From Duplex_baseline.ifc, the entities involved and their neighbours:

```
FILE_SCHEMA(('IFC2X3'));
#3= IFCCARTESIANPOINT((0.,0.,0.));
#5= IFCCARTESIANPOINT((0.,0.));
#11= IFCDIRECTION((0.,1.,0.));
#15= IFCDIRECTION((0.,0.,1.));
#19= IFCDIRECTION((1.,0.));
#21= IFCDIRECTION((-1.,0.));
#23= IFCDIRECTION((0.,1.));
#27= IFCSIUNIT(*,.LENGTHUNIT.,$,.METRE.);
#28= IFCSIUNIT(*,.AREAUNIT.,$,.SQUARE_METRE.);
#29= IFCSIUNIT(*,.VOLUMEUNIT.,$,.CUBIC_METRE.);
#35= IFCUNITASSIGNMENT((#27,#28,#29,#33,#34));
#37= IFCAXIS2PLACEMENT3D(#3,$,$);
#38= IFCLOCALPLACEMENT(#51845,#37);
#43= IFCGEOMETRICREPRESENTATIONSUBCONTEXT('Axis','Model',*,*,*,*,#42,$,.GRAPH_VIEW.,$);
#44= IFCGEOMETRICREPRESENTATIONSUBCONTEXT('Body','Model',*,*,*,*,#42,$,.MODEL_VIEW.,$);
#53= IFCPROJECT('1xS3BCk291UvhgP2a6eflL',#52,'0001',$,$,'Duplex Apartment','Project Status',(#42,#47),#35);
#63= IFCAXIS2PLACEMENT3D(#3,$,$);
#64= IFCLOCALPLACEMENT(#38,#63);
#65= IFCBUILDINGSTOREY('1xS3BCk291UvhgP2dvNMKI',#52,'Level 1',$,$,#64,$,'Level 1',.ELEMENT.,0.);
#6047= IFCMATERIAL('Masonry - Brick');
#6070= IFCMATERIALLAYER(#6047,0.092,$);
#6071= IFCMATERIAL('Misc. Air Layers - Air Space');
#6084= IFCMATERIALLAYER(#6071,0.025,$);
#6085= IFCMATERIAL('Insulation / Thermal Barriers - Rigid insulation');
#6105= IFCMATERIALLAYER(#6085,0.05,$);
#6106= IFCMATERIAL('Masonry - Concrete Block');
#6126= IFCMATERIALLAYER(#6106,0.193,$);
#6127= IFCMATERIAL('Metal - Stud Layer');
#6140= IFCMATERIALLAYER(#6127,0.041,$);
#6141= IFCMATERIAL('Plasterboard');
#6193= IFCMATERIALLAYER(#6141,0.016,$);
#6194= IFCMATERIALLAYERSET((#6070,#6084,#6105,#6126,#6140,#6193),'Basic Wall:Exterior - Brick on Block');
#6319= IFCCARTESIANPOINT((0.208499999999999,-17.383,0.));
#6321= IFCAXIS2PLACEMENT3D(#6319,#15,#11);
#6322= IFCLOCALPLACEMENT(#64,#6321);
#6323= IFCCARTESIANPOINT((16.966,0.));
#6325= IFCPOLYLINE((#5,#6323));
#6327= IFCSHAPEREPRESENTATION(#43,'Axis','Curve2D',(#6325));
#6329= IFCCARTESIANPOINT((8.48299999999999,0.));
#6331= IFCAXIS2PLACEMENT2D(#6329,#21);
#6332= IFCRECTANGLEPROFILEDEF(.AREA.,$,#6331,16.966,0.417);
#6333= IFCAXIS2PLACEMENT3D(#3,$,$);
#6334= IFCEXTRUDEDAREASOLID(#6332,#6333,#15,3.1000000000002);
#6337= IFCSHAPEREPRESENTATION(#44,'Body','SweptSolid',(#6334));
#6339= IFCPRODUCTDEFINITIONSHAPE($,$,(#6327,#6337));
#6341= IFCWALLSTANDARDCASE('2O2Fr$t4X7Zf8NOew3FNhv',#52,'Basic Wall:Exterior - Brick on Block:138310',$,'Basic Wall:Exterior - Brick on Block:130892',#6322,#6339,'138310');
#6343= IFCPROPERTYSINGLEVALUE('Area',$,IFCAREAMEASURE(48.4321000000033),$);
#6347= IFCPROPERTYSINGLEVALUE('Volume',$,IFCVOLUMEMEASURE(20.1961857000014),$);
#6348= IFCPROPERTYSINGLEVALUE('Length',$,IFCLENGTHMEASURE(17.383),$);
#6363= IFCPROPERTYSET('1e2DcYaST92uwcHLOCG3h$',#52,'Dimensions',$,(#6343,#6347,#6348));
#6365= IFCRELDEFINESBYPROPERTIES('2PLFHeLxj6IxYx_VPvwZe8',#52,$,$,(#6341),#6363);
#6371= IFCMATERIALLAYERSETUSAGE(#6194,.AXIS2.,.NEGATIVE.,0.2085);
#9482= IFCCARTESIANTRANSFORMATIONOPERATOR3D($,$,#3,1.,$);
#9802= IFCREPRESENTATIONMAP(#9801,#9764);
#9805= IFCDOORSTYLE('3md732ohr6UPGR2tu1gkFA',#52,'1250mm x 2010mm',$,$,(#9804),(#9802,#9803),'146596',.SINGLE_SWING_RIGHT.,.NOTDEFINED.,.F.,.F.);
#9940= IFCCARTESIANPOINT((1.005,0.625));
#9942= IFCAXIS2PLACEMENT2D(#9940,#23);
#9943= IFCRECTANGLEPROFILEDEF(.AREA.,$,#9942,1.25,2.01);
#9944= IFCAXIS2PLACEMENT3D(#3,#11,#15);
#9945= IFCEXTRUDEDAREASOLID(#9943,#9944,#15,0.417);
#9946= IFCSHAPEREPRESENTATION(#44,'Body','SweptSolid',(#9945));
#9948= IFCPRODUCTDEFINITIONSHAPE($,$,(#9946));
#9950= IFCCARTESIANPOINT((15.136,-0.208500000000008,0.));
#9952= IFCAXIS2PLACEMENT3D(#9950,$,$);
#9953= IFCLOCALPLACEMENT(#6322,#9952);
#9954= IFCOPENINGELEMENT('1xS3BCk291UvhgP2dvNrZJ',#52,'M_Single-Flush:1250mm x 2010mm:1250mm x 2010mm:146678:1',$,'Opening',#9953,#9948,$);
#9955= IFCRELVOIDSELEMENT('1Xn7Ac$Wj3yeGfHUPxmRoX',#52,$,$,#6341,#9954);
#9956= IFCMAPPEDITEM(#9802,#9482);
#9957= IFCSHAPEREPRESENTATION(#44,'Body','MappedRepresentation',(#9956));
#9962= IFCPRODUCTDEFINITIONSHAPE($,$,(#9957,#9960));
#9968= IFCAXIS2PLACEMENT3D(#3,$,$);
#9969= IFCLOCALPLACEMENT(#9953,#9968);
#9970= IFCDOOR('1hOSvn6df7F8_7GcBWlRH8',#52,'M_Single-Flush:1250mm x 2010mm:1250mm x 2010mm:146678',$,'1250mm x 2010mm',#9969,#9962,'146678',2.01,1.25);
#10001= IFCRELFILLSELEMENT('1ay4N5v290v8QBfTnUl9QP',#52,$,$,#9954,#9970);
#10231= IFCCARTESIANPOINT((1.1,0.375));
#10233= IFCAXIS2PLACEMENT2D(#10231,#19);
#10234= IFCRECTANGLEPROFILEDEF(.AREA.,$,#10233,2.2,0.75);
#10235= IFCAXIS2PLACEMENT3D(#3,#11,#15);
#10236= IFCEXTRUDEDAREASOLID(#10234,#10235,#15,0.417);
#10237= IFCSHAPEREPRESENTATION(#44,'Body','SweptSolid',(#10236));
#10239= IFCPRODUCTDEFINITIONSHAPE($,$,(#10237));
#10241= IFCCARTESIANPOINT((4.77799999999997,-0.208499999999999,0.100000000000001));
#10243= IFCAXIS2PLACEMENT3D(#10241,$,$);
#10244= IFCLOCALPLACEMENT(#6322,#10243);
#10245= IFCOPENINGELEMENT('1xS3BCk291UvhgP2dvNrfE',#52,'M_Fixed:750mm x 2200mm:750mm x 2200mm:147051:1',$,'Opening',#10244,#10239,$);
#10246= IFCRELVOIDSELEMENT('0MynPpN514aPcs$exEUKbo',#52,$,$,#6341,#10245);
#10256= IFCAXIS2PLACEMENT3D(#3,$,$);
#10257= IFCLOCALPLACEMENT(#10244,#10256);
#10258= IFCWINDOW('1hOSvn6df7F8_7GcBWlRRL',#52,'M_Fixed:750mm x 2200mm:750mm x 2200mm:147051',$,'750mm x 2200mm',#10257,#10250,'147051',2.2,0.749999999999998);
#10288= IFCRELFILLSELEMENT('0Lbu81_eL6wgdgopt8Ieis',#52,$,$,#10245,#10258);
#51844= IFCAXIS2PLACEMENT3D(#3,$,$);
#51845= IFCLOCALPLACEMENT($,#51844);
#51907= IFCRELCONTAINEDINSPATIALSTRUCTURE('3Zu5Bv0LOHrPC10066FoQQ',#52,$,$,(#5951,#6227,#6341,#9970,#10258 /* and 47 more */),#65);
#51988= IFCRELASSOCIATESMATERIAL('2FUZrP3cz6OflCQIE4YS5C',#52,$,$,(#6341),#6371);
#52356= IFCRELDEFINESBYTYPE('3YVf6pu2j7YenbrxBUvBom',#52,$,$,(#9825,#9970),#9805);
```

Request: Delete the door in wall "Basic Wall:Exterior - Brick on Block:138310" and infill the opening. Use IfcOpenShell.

```python
import ifcopenshell
import ifcopenshell.api.feature
import ifcopenshell.api.pset
import ifcopenshell.api.root
import ifcopenshell.geom
import ifcopenshell.util.element
import ifcopenshell.util.shape
import ifcopenshell.util.unit

model = ifcopenshell.open("Duplex_baseline.ifc")
area_scale = ifcopenshell.util.unit.calculate_unit_scale(model, "AREAUNIT")
volume_scale = ifcopenshell.util.unit.calculate_unit_scale(model, "VOLUMEUNIT")
settings = ifcopenshell.geom.settings()


def volume(element):
    """Net volume in cubic metres, openings subtracted."""
    shape = ifcopenshell.geom.create_shape(settings, element)
    return ifcopenshell.util.shape.get_volume(shape.geometry)


door = model.by_id(9970)
opening = door.FillsVoids[0].RelatingOpeningElement
wall = opening.VoidsElements[0].RelatingBuildingElement
before = volume(wall)

ifcopenshell.api.root.remove_product(model, product=door)
ifcopenshell.api.feature.remove_feature(model, feature=opening)

after = volume(wall)
thickness = 0.417  # wall thickness in metres

# Update the wall's stored quantities.
pset = model.by_id(ifcopenshell.util.element.get_pset(wall, "Dimensions", should_inherit=False)["id"])
ifcopenshell.api.pset.edit_pset(model, pset=pset, properties={
    "Area": model.create_entity("IfcAreaMeasure", after / thickness / area_scale),
    "Volume": model.create_entity("IfcVolumeMeasure", after / volume_scale),
})

print(f"wall volume {before:.3f} -> {after:.3f} m3")

model.write("Duplex_baseline_edited.ifc")
```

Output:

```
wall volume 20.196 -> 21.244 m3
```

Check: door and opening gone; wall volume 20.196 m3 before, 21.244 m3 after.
